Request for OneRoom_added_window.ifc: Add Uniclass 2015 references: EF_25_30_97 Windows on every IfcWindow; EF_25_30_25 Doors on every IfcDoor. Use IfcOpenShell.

First a look at what the model holds.

```python
import ifcopenshell

model = ifcopenshell.open("OneRoom_added_window.ifc")
print(model.schema)
print("classifications:", [c.Name for c in model.by_type("IfcClassification")])
for ifc_class in ("IfcDoor", "IfcRoof", "IfcStair", "IfcWall", "IfcWindow"):
    print(ifc_class, len(model.by_type(ifc_class)))
```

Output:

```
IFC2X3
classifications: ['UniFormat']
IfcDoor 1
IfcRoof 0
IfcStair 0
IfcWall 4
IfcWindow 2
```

```python
import ifcopenshell
import ifcopenshell.api.classification

model = ifcopenshell.open("OneRoom_added_window.ifc")

# IFC2X3 requires Source and Edition and has no link from the project to the system.
system = model.create_entity("IfcClassification", Source="NBS", Edition="2015", Name="Uniclass 2015")

codes = {
    "IfcWindow": ("EF_25_30_97", "Windows"),
    "IfcDoor": ("EF_25_30_25", "Doors"),
}
for ifc_class, (code, name) in codes.items():
    products = model.by_type(ifc_class)
    ifcopenshell.api.classification.add_reference(
        model, products=products, classification=system, identification=code, name=name
    )
    print(code, len(products))

model.write("OneRoom_added_window_rev.ifc")
```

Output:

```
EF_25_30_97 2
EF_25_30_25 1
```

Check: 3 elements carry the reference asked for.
